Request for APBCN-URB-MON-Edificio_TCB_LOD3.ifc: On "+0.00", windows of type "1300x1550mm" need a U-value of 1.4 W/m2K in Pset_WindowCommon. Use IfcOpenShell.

First a look at what the model holds.

```python
import ifcopenshell
import ifcopenshell.util.element

model = ifcopenshell.open("APBCN-URB-MON-Edificio_TCB_LOD3.ifc")
print(model.schema)
storey = next(s for s in model.by_type("IfcBuildingStorey") if s.Name == "+0.00")
windows = [e for e in ifcopenshell.util.element.get_decomposition(storey) if e.is_a("IfcWindow")]
seen = {}
for e in windows:
    element_type = ifcopenshell.util.element.get_type(e)
    key = (element_type.Name if element_type != e and element_type else None, ifcopenshell.util.element.get_pset(e, "Pset_WindowCommon", "ThermalTransmittance"))
    seen[key] = seen.get(key, 0) + 1
for (name, value), count in sorted(seen.items(), key=str):
    print(count, "x", name, "|", value)
```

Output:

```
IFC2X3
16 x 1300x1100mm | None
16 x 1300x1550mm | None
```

```python
import ifcopenshell
import ifcopenshell.api.pset
import ifcopenshell.util.element

model = ifcopenshell.open("APBCN-URB-MON-Edificio_TCB_LOD3.ifc")

storey = next(s for s in model.by_type("IfcBuildingStorey") if s.Name == "+0.00")
windows = [e for e in ifcopenshell.util.element.get_decomposition(storey) if e.is_a("IfcWindow")]

count = 0
for e in windows:
    element_type = ifcopenshell.util.element.get_type(e)
    if element_type in (None, e) or element_type.Name != "1300x1550mm":
        continue
    # add_pset returns the element's existing set when there is one.
    pset = ifcopenshell.api.pset.add_pset(model, product=e, name="Pset_WindowCommon")
    ifcopenshell.api.pset.edit_pset(model, pset=pset, properties={"ThermalTransmittance": 1.4})
    count += 1

print(count, "windows updated")

model.write("APBCN-URB-MON-Edificio_TCB_LOD3_updated.ifc")
```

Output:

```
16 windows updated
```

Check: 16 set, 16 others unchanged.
